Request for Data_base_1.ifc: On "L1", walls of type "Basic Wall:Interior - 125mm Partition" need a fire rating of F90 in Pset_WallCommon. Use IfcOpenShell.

First a look at what the model holds.

```python
import ifcopenshell
import ifcopenshell.util.element

model = ifcopenshell.open("Data_base_1.ifc")
print(model.schema)
storey = next(s for s in model.by_type("IfcBuildingStorey") if s.Name == "L1")
walls = [e for e in ifcopenshell.util.element.get_decomposition(storey) if e.is_a("IfcWall")]
seen = {}
for e in walls:
    element_type = ifcopenshell.util.element.get_type(e)
    key = (element_type.Name if element_type != e and element_type else None, ifcopenshell.util.element.get_pset(e, "Pset_WallCommon", "FireRating"))
    seen[key] = seen.get(key, 0) + 1
for (name, value), count in sorted(seen.items(), key=str):
    print(count, "x", name, "|", value)
```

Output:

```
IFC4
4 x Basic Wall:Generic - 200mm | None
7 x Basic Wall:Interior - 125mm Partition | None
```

```python
import ifcopenshell
import ifcopenshell.api.pset
import ifcopenshell.util.element

model = ifcopenshell.open("Data_base_1.ifc")

storey = next(s for s in model.by_type("IfcBuildingStorey") if s.Name == "L1")
walls = [e for e in ifcopenshell.util.element.get_decomposition(storey) if e.is_a("IfcWall")]

count = 0
for e in walls:
    element_type = ifcopenshell.util.element.get_type(e)
    if element_type in (None, e) or element_type.Name != "Basic Wall:Interior - 125mm Partition":
        continue
    # add_pset returns the element's existing set when there is one.
    pset = ifcopenshell.api.pset.add_pset(model, product=e, name="Pset_WallCommon")
    ifcopenshell.api.pset.edit_pset(model, pset=pset, properties={"FireRating": "F90"})
    count += 1

print(count, "walls updated")

model.write("Data_base_1-out.ifc")
```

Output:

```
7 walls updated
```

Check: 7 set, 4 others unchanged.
